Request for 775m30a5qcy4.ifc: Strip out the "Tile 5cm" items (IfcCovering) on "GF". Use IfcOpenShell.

First a look at what the model holds.

```python
import ifcopenshell
import ifcopenshell.util.element

model = ifcopenshell.open("775m30a5qcy4.ifc")
print(model.schema)
storey = next(s for s in model.by_type("IfcBuildingStorey") if s.Name == "GF")
coverings = [e for e in ifcopenshell.util.element.get_decomposition(storey) if e.is_a("IfcCovering")]
seen = {}
for e in coverings:
    element_type = ifcopenshell.util.element.get_type(e)
    name = element_type.Name if element_type not in (None, e) else None
    seen[name] = seen.get(name, 0) + 1
for name, count in sorted(seen.items(), key=str):
    print(count, "x", name)
```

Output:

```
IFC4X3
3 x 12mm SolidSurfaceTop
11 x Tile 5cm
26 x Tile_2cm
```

```python
import ifcopenshell
import ifcopenshell.api.root
import ifcopenshell.util.element

model = ifcopenshell.open("775m30a5qcy4.ifc")

storey = next(s for s in model.by_type("IfcBuildingStorey") if s.Name == "GF")
coverings = [e for e in ifcopenshell.util.element.get_decomposition(storey) if e.is_a("IfcCovering")]
targets = [e for e in coverings if (t := ifcopenshell.util.element.get_type(e)) not in (None, e) and t.Name == "Tile 5cm"]

for e in targets:
    ifcopenshell.api.root.remove_product(model, product=e)
print(len(targets), "removed")

model.write("775m30a5qcy4_updated.ifc")
```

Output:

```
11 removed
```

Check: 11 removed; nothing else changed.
